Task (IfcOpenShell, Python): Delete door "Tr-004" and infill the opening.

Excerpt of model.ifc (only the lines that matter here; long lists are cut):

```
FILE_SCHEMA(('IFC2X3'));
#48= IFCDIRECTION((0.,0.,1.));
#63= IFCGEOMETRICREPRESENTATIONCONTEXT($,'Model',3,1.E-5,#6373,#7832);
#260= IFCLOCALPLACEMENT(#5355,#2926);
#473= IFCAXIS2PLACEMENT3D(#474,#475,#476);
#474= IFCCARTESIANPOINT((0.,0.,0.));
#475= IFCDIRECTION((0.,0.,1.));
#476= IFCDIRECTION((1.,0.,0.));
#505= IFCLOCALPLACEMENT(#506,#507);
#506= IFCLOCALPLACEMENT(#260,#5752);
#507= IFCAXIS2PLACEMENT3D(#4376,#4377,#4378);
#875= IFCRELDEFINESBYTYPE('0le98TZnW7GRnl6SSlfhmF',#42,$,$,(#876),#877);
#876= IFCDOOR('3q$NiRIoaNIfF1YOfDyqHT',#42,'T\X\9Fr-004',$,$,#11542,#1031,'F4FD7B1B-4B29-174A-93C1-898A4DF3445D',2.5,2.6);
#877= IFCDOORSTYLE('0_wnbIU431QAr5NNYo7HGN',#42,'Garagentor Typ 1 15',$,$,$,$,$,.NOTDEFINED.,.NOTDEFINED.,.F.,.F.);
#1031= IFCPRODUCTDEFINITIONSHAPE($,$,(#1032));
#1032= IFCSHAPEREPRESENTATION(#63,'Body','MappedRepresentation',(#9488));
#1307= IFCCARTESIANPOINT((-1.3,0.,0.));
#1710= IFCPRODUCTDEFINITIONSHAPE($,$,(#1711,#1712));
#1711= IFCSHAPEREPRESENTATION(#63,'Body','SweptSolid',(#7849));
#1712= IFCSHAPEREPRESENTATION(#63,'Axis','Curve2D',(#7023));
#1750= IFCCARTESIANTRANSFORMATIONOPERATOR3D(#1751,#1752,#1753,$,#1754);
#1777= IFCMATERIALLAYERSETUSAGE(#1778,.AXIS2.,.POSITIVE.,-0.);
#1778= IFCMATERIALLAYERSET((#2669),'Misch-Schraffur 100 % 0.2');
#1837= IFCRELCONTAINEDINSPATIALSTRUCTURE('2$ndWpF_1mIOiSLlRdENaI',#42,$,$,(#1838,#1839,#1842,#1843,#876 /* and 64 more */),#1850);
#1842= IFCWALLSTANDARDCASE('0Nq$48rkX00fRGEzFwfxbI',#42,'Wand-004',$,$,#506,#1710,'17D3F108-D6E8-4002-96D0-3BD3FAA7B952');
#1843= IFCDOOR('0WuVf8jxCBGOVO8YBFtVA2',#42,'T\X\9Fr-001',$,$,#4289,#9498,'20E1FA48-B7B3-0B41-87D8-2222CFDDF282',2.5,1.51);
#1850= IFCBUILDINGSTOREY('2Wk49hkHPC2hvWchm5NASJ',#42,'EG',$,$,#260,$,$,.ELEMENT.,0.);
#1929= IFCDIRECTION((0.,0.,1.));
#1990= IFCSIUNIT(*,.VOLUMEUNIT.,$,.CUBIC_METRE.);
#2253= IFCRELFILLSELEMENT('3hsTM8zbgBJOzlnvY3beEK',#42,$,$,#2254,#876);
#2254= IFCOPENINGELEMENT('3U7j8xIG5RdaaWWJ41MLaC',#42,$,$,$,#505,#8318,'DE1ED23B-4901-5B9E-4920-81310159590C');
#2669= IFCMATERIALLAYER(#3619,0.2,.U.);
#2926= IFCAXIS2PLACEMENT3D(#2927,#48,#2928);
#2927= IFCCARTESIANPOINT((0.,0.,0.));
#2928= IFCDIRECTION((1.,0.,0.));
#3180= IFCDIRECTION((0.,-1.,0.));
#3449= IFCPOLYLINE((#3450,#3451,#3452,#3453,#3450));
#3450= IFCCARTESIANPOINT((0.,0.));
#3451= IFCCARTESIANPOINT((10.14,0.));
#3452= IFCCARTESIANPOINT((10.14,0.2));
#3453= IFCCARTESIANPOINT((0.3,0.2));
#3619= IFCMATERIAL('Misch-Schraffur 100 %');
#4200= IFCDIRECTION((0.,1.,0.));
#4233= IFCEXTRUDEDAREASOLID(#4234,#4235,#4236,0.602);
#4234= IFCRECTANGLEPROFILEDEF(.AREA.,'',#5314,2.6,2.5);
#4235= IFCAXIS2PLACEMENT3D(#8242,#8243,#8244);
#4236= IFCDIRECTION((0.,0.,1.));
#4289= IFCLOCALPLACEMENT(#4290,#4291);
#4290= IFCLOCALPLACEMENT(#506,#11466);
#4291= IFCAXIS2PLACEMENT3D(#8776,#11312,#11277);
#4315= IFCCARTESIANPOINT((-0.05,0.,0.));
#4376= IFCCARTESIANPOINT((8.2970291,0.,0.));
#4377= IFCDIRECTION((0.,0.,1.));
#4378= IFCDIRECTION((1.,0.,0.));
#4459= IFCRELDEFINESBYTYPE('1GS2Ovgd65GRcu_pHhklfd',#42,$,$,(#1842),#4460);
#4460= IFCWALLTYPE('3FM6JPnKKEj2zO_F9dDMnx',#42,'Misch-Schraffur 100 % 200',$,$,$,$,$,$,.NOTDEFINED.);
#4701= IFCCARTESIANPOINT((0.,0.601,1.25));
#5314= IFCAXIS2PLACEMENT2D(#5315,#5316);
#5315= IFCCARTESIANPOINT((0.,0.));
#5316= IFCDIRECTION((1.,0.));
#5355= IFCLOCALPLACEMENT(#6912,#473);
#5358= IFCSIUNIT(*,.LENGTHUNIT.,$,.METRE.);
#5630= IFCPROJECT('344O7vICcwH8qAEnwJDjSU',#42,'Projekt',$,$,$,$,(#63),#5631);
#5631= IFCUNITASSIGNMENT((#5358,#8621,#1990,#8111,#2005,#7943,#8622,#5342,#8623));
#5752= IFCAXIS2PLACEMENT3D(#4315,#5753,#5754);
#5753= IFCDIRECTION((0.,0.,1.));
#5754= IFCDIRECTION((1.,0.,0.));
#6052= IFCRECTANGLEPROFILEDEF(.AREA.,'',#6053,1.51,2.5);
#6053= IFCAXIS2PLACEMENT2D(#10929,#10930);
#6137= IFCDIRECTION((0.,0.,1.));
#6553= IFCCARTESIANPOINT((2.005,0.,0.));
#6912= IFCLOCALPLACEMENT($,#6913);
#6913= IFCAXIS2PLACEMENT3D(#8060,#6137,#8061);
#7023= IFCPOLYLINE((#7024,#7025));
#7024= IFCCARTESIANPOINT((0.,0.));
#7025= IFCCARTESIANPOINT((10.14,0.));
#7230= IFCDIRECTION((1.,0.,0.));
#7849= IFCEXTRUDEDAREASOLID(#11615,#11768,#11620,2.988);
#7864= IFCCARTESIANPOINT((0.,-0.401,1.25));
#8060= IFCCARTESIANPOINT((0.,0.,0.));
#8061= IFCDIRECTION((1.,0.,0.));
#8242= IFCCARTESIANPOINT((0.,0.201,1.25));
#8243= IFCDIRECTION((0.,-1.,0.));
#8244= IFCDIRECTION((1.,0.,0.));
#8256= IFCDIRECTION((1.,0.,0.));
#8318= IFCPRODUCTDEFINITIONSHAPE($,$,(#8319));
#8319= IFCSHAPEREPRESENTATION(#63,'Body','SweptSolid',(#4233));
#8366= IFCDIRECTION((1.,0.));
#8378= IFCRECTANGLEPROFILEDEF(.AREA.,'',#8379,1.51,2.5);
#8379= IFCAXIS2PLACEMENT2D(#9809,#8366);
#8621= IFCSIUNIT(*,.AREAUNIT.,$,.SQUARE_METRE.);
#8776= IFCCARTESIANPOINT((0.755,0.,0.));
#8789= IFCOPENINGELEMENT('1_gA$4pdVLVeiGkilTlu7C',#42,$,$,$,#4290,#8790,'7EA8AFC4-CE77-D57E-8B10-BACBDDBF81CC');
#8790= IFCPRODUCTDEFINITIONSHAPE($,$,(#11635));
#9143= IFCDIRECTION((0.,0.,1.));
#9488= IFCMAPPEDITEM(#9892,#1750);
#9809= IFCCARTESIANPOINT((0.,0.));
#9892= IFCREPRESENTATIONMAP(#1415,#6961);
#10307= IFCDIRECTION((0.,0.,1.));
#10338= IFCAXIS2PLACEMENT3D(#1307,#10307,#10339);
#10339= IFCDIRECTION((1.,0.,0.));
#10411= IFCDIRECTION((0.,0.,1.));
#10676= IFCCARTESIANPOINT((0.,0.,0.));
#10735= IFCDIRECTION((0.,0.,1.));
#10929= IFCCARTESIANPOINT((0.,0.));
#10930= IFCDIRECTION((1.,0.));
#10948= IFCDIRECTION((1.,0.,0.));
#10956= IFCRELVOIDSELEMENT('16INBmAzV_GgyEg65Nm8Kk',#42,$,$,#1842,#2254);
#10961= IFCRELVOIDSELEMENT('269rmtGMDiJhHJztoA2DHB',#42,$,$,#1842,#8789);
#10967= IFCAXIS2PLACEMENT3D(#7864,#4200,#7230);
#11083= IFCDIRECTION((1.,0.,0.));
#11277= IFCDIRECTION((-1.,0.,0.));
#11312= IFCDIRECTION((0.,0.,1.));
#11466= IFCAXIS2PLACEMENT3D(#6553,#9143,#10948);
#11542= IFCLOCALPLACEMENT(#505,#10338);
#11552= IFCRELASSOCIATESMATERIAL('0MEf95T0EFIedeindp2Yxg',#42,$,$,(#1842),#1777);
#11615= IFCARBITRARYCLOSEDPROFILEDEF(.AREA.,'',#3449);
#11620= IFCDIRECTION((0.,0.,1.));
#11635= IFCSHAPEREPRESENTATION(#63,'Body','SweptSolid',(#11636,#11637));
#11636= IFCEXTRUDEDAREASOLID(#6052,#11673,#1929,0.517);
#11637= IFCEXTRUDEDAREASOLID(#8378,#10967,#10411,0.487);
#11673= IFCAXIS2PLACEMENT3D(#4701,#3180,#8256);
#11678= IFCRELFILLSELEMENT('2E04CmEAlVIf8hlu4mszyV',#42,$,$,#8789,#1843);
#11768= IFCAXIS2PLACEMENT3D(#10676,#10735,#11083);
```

```python
import ifcopenshell
import ifcopenshell.api.feature
import ifcopenshell.api.root
import ifcopenshell.geom
import ifcopenshell.util.shape

model = ifcopenshell.open("model.ifc")
settings = ifcopenshell.geom.settings()


def volume(element):
    """Net volume in cubic metres, openings subtracted."""
    shape = ifcopenshell.geom.create_shape(settings, element)
    return ifcopenshell.util.shape.get_volume(shape.geometry)


door = model.by_id(876)
opening = door.FillsVoids[0].RelatingOpeningElement
wall = opening.VoidsElements[0].RelatingBuildingElement
before = volume(wall)

ifcopenshell.api.root.remove_product(model, product=door)
ifcopenshell.api.feature.remove_feature(model, feature=opening)

after = volume(wall)

print(f"wall volume {before:.3f} -> {after:.3f} m3")

model.write("model-out.ifc")
```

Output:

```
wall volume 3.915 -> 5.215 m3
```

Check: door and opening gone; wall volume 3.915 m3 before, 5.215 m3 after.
